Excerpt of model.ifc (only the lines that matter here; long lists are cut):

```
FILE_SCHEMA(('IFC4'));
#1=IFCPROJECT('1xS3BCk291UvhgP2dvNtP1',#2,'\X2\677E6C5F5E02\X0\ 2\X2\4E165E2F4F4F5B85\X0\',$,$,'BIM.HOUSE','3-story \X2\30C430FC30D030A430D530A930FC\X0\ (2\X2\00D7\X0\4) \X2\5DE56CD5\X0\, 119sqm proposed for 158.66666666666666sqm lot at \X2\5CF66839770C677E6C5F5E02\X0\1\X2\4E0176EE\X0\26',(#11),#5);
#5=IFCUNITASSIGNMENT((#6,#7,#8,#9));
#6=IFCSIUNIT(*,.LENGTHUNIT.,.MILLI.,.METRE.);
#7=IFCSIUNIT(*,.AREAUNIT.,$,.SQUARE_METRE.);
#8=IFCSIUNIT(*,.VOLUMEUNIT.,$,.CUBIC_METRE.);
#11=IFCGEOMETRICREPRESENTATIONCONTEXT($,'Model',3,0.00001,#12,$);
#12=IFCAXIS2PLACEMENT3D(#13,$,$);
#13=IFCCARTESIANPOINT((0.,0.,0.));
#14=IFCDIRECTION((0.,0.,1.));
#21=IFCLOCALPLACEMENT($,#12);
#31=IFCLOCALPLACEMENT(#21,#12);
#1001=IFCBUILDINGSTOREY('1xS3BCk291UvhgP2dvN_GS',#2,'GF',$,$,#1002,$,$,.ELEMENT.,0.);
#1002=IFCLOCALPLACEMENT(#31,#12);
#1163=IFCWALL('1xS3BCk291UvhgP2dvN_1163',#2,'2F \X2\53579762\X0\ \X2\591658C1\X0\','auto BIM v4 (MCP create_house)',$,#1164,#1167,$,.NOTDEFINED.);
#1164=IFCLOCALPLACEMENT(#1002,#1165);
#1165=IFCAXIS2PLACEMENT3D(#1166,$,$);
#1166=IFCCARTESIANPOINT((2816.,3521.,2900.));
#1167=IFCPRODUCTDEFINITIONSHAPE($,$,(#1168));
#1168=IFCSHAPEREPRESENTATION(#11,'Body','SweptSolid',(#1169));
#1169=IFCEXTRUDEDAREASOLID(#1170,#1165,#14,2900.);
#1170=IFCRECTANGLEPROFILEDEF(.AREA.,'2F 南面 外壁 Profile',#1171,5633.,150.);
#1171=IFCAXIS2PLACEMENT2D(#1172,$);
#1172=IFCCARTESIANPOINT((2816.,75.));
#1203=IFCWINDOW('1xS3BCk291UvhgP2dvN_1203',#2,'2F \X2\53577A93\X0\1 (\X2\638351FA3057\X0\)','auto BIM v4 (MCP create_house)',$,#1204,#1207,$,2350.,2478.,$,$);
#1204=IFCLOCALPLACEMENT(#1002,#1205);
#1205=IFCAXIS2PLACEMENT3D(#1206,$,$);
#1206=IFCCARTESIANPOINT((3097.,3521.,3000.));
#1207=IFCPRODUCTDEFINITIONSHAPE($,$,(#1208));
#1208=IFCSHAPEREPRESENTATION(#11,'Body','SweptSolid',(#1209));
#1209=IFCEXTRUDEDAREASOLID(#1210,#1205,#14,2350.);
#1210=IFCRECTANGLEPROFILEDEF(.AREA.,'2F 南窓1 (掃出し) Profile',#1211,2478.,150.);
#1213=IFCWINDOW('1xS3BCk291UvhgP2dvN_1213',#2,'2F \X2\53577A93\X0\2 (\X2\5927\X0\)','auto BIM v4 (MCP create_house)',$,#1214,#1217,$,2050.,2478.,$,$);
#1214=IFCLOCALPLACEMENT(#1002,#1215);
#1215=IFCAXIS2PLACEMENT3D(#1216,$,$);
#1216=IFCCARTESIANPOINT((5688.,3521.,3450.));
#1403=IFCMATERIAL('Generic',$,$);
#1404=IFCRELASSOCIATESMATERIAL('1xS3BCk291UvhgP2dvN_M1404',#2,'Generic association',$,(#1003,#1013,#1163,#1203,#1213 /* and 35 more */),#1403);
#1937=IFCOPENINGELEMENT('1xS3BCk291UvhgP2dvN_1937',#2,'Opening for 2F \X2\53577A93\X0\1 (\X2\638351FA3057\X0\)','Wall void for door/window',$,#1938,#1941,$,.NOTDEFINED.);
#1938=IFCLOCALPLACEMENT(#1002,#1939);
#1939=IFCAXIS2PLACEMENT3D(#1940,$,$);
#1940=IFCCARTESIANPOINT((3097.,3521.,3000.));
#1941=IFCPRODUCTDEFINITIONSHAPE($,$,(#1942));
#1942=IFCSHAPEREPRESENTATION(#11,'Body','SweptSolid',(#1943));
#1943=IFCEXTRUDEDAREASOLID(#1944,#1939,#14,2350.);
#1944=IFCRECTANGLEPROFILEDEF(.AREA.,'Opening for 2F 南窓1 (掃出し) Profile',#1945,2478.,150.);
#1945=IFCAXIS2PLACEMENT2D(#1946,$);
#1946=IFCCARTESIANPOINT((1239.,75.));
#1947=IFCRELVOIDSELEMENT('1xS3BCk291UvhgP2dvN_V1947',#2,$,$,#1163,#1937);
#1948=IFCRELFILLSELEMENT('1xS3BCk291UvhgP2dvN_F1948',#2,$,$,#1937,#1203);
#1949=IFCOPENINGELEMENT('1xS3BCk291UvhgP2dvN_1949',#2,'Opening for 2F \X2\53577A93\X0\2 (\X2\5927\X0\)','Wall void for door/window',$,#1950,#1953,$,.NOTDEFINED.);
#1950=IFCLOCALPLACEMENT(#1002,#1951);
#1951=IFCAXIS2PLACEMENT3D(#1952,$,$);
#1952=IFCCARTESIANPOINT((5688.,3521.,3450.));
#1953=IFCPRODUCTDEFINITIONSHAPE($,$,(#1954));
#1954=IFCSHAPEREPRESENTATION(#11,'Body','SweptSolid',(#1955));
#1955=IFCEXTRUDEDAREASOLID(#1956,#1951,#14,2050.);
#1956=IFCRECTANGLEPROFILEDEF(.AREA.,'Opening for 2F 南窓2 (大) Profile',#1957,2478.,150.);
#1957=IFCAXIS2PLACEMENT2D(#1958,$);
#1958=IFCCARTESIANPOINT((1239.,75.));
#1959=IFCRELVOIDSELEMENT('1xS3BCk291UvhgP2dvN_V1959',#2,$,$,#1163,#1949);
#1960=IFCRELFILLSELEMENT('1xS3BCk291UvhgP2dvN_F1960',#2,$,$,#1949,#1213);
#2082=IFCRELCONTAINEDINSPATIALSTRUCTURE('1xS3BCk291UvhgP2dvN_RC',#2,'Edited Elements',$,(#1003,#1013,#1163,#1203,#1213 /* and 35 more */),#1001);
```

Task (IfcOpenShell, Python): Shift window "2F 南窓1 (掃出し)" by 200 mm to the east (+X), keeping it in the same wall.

```python
import ifcopenshell
import ifcopenshell.api.geometry
import ifcopenshell.util.placement
import ifcopenshell.util.unit

model = ifcopenshell.open("model.ifc")
unit_scale = ifcopenshell.util.unit.calculate_unit_scale(model)

window = model.by_id(1203)
opening = window.FillsVoids[0].RelatingOpeningElement
wall = opening.VoidsElements[0].RelatingBuildingElement

wall_matrix = ifcopenshell.util.placement.get_local_placement(wall.ObjectPlacement)
shift = wall_matrix[:3, 0] * 0.2 / unit_scale
before = ifcopenshell.util.placement.get_local_placement(window.ObjectPlacement)[:3, 3].copy()

# The window is not placed relative to its opening, so move both.
for product in (opening, window):
    matrix = ifcopenshell.util.placement.get_local_placement(product.ObjectPlacement)
    matrix[:3, 3] += shift
    ifcopenshell.api.geometry.edit_object_placement(model, product=product, matrix=matrix, is_si=False)

after = ifcopenshell.util.placement.get_local_placement(window.ObjectPlacement)[:3, 3]
print("window moved by", (after - before).round(3) + 0.0)

model.write("model_rev.ifc")
```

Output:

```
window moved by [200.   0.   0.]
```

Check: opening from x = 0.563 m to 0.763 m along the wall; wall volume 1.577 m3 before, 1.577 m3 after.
